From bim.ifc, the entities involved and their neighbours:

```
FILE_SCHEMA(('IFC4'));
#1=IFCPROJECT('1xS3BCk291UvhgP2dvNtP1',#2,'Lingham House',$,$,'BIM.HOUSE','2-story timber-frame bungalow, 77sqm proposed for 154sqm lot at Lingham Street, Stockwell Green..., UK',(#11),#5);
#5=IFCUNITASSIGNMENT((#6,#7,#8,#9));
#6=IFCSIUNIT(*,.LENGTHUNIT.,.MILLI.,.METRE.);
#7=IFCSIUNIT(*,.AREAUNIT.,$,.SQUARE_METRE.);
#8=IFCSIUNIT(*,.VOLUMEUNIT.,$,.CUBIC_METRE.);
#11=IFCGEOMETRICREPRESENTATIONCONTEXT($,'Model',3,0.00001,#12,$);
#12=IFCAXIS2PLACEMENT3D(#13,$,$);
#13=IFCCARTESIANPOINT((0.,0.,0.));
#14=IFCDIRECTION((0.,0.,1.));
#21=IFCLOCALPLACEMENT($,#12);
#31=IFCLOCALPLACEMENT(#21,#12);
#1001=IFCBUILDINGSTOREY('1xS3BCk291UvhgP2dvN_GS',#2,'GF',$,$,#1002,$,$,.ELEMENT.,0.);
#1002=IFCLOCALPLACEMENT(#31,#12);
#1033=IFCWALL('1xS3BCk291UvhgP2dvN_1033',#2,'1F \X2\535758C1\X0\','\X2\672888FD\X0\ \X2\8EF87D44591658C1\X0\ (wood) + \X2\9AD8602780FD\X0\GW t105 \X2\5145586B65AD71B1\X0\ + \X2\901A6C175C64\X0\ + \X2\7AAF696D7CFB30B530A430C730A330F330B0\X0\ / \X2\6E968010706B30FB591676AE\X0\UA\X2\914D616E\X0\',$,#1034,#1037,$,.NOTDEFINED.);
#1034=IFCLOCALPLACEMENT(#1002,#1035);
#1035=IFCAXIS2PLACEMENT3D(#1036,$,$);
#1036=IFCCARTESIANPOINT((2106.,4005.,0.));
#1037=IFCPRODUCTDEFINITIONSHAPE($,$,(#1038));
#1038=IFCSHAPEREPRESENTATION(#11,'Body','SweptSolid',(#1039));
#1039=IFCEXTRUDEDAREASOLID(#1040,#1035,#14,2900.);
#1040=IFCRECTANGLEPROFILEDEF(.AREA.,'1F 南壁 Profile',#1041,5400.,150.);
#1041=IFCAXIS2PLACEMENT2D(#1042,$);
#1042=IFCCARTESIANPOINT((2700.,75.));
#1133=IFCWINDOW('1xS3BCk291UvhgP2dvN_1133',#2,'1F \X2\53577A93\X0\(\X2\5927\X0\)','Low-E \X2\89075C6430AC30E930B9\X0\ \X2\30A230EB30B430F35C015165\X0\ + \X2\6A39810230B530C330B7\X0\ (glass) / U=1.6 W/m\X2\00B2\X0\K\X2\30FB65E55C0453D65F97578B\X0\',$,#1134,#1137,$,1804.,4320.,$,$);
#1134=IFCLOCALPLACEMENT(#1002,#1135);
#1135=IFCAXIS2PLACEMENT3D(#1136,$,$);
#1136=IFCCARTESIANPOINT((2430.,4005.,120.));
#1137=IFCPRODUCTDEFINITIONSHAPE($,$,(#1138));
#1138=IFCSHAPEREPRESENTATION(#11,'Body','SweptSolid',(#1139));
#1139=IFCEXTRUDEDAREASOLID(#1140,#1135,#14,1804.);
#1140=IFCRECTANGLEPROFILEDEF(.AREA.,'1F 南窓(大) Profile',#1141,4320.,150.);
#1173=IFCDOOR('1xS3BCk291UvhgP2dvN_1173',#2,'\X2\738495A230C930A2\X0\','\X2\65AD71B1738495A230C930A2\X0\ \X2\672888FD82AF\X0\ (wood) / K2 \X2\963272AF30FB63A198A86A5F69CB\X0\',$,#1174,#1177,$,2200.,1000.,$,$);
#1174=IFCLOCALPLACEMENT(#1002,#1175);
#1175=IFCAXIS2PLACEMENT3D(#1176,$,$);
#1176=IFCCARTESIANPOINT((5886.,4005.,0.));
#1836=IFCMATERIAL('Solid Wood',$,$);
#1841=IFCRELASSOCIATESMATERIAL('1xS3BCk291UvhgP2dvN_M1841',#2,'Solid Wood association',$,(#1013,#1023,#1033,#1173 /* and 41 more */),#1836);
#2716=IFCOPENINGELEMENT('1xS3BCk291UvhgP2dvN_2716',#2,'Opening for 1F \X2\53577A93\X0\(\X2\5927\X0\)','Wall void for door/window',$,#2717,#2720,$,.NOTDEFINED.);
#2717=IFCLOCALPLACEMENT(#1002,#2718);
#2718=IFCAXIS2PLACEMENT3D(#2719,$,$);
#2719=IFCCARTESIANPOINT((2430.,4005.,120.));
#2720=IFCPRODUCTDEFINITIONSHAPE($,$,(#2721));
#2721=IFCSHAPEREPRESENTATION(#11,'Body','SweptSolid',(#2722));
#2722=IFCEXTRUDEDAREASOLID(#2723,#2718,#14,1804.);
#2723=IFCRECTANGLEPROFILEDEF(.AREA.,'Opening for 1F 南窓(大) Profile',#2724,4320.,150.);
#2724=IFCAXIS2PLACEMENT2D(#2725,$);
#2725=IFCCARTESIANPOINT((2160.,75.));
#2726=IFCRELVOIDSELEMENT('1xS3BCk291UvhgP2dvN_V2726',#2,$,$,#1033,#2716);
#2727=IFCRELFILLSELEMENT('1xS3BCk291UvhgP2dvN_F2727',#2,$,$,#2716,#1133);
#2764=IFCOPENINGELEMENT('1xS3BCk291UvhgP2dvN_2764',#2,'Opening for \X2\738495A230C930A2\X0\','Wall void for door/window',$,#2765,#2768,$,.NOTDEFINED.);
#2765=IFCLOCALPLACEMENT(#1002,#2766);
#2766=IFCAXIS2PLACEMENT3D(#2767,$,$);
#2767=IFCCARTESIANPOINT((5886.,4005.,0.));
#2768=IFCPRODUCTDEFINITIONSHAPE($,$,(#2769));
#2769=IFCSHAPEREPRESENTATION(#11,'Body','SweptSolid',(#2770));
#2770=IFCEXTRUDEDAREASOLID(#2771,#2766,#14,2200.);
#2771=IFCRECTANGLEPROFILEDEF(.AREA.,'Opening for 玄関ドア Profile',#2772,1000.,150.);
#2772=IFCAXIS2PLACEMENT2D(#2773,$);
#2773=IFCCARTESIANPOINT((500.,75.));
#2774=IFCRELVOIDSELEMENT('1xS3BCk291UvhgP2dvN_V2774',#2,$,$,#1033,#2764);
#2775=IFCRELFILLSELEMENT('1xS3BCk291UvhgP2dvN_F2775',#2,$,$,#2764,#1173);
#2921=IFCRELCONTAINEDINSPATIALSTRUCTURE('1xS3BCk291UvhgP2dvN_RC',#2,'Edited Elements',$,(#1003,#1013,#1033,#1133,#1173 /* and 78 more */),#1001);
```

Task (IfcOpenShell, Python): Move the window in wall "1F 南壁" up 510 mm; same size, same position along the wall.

```python
import numpy as np
import ifcopenshell
import ifcopenshell.api.geometry
import ifcopenshell.util.placement
import ifcopenshell.util.unit

model = ifcopenshell.open("bim.ifc")
unit_scale = ifcopenshell.util.unit.calculate_unit_scale(model)

window = model.by_id(1133)
opening = window.FillsVoids[0].RelatingOpeningElement
dz = 0.51 / unit_scale

shift = np.array([0.0, 0.0, dz])
# The window is not placed relative to its opening, so move both.
for product in (opening, window):
    matrix = ifcopenshell.util.placement.get_local_placement(product.ObjectPlacement)
    matrix[:3, 3] += shift
    ifcopenshell.api.geometry.edit_object_placement(model, product=product, matrix=matrix, is_si=False)

print(f"moved by {dz * unit_scale:+.3f} m")

model.write("bim_rev.ifc")
```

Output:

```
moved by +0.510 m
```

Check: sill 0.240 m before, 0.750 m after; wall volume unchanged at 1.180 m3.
